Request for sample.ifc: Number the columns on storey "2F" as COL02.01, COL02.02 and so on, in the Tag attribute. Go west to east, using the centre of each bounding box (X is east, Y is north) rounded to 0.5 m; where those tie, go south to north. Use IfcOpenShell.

First a look at what the model holds.

```python
import ifcopenshell
import ifcopenshell.util.element
import ifcopenshell.util.placement

model = ifcopenshell.open("sample.ifc")
print(model.schema)
storey = next(s for s in model.by_type("IfcBuildingStorey") if s.Name == "2F")
columns = [e for e in ifcopenshell.util.element.get_decomposition(storey) if e.is_a("IfcColumn")]
for e in sorted(columns, key=lambda e: e.id()):
    origin = ifcopenshell.util.placement.get_local_placement(e.ObjectPlacement)[:3, 3]
    print(e.id(), e.Tag, e.Name, origin.round(2) + 0.0, sep=" | ")
```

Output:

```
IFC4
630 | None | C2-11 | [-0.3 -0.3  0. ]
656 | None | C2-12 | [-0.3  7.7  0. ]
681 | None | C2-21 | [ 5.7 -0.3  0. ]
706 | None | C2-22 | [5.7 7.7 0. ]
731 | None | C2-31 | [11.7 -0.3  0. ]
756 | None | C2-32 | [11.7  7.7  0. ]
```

```python
import ifcopenshell
import ifcopenshell.geom
import ifcopenshell.util.element
import ifcopenshell.util.shape

model = ifcopenshell.open("sample.ifc")
settings = ifcopenshell.geom.settings()
settings.set("use-world-coords", True)


def centre(element):
    shape = ifcopenshell.geom.create_shape(settings, element)
    return ifcopenshell.util.shape.get_bbox_centroid(shape.geometry)


storey = next(s for s in model.by_type("IfcBuildingStorey") if s.Name == "2F")
columns = [e for e in ifcopenshell.util.element.get_decomposition(storey) if e.is_a("IfcColumn")]

# Insertion points can sit at a corner or the storey origin, so sort by the geometry (in metres).
centres = {e: centre(e) for e in columns}
columns.sort(key=lambda e: (round(centres[e][0] / 0.5), centres[e][1]))

for i, e in enumerate(columns, start=1):
    number = f"COL02.{i:02d}"
    e.Tag = number
    print(e.id(), number)

model.write("sample_v2.ifc")
```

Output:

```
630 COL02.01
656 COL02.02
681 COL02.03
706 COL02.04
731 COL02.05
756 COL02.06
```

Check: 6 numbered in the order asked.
